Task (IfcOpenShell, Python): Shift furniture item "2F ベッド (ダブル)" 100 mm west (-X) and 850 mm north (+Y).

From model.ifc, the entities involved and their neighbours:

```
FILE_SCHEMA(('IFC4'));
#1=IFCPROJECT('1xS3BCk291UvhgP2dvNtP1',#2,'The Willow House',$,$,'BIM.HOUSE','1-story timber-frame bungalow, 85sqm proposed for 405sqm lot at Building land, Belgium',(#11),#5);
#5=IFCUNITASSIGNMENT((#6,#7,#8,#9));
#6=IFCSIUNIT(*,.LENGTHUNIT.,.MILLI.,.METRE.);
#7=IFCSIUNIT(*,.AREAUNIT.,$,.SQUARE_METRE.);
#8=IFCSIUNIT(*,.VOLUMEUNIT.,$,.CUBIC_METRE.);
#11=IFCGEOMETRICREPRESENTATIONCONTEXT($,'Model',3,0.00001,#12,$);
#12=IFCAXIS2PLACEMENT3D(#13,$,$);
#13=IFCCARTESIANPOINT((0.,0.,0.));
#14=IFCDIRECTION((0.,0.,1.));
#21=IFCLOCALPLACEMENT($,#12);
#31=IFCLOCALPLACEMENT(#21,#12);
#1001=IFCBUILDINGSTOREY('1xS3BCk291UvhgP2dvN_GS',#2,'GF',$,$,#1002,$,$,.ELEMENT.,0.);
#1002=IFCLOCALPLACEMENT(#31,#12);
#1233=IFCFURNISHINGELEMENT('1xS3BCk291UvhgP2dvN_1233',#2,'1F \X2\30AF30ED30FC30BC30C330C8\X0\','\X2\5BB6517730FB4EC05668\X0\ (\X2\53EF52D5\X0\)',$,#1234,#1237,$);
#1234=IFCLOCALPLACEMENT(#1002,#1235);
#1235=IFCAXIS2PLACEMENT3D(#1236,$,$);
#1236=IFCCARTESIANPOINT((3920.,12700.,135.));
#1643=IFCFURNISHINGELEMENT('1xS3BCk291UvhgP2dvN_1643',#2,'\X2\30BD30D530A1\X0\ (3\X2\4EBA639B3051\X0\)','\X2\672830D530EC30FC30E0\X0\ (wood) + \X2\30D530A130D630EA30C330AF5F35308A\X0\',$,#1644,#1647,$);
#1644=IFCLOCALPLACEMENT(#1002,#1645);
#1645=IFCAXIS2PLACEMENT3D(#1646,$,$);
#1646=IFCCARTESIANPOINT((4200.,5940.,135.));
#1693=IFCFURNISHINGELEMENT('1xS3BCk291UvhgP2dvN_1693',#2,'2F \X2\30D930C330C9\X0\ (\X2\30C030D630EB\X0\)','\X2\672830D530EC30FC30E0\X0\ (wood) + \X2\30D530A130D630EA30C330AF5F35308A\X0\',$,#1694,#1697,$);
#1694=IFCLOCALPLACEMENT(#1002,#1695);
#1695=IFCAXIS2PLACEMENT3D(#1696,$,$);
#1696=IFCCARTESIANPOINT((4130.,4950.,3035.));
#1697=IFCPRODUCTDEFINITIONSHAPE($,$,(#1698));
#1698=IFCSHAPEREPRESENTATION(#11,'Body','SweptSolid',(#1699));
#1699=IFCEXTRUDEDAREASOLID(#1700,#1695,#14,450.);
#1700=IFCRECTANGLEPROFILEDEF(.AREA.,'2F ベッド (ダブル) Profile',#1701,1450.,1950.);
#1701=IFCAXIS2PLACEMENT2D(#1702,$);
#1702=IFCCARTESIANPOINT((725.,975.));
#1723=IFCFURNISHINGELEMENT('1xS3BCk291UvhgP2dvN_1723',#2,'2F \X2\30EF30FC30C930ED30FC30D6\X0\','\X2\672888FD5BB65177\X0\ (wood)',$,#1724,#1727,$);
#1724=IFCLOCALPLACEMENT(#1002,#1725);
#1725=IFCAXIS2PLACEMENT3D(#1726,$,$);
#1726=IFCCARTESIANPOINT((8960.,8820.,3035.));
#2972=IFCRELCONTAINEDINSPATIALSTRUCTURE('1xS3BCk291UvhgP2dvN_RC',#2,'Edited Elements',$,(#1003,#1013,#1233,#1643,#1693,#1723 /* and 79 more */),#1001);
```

```python
import ifcopenshell
import ifcopenshell.api.geometry
import ifcopenshell.util.placement
import ifcopenshell.util.unit

model = ifcopenshell.open("model.ifc")
unit_scale = ifcopenshell.util.unit.calculate_unit_scale(model)

item = model.by_guid("1xS3BCk291UvhgP2dvN_1693")
matrix = ifcopenshell.util.placement.get_local_placement(item.ObjectPlacement)
matrix[0, 3] -= 0.1 / unit_scale
matrix[1, 3] += 0.85 / unit_scale
ifcopenshell.api.geometry.edit_object_placement(model, product=item, matrix=matrix, is_si=False)

print(ifcopenshell.util.placement.get_local_placement(item.ObjectPlacement).round(3) + 0.0)

model.write("model_v2.ifc")
```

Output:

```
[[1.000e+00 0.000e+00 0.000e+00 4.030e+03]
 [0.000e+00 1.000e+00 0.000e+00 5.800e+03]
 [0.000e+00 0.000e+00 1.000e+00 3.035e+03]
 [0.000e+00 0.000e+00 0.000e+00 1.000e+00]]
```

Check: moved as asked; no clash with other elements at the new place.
